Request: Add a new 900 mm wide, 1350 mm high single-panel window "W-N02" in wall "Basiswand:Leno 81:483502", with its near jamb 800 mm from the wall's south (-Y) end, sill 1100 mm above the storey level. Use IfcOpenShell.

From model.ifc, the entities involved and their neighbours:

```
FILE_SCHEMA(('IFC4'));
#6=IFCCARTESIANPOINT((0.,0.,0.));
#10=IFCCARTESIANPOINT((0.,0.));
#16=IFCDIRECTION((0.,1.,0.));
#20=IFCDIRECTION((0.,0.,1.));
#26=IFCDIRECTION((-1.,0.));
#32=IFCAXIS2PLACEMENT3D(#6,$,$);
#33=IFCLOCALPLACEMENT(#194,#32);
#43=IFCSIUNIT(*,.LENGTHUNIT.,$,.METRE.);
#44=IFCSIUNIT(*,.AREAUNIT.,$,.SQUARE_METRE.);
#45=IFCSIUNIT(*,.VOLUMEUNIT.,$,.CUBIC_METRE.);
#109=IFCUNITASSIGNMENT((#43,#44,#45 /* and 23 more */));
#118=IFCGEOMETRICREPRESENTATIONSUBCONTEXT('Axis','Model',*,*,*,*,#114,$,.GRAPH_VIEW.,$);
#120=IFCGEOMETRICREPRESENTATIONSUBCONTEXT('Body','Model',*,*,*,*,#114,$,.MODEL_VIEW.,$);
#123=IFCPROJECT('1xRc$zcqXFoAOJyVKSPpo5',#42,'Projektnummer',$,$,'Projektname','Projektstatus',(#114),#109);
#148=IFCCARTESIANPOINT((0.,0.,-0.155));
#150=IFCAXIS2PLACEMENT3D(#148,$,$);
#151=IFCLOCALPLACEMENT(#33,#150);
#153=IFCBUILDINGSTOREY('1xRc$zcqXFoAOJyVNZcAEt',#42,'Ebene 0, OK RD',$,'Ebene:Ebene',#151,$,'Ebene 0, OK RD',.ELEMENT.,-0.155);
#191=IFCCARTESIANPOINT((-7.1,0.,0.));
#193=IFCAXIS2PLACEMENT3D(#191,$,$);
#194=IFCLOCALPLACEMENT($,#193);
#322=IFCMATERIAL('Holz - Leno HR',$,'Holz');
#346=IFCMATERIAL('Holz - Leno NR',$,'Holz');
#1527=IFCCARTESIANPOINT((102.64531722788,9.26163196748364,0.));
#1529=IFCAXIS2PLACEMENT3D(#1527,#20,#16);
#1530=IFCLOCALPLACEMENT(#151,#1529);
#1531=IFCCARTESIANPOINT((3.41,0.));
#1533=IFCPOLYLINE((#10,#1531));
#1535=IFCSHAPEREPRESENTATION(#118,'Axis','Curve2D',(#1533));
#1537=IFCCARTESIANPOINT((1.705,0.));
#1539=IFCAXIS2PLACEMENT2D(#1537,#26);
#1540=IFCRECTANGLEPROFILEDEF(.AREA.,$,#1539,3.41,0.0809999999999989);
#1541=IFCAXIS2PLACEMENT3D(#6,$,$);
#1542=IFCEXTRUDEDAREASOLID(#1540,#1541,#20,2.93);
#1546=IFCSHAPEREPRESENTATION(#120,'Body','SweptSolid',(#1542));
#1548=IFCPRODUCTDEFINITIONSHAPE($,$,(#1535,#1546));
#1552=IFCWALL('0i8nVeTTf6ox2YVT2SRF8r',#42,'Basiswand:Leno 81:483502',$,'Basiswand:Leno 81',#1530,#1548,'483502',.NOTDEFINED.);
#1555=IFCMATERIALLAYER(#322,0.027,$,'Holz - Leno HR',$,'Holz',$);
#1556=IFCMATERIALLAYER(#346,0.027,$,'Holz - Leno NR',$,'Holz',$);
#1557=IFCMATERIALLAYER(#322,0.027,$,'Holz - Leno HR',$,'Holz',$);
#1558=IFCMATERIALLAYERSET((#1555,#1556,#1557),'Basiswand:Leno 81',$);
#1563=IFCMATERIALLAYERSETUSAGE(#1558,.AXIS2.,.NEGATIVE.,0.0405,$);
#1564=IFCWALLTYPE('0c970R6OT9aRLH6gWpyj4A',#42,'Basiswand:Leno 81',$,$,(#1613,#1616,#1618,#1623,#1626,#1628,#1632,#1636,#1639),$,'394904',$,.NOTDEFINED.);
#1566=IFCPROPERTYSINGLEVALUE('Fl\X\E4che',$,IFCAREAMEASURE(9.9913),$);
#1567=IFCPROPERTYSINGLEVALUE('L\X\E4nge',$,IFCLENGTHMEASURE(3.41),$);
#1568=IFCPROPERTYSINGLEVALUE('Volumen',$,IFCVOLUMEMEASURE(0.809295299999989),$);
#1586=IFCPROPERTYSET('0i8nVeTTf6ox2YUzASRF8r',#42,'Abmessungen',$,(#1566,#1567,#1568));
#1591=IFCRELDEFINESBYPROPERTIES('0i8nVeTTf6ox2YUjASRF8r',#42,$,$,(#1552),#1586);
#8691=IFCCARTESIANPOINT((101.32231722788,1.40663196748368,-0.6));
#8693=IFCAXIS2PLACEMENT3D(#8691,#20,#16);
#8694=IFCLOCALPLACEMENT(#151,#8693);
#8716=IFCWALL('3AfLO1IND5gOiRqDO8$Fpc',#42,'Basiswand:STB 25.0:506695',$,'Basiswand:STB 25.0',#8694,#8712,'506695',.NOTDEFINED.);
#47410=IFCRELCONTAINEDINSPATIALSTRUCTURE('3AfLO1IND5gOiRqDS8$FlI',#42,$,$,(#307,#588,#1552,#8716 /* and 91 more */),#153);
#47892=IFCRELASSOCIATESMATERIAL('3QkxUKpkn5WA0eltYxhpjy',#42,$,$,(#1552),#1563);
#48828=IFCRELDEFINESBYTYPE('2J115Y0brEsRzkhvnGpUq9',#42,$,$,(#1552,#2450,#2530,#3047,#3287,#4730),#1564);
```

```python
import numpy as np
import ifcopenshell
import ifcopenshell.api.feature
import ifcopenshell.api.geometry
import ifcopenshell.api.pset
import ifcopenshell.api.root
import ifcopenshell.api.spatial
import ifcopenshell.geom
import ifcopenshell.util.element
import ifcopenshell.util.placement
import ifcopenshell.util.representation
import ifcopenshell.util.shape
import ifcopenshell.util.unit

model = ifcopenshell.open("model.ifc")
unit_scale = ifcopenshell.util.unit.calculate_unit_scale(model)
area_scale = ifcopenshell.util.unit.calculate_unit_scale(model, "AREAUNIT")
volume_scale = ifcopenshell.util.unit.calculate_unit_scale(model, "VOLUMEUNIT")
settings = ifcopenshell.geom.settings()


def volume(element):
    """Net volume in cubic metres, openings subtracted."""
    shape = ifcopenshell.geom.create_shape(settings, element)
    return ifcopenshell.util.shape.get_volume(shape.geometry)


wall = model.by_id(1552)
storey = ifcopenshell.util.element.get_container(wall, ifc_class="IfcBuildingStorey")
context = ifcopenshell.util.representation.get_context(model, "Model", "Body", "MODEL_VIEW")
before = volume(wall)

width, height, from_end, sill = 0.9, 1.35, 0.8, 1.1  # metres

# The wall runs along its own X axis, and the end named is its -X end.
wall_shape = ifcopenshell.geom.create_shape(settings, wall)
x, y, z = ifcopenshell.util.shape.get_vertices(wall_shape.geometry).T
start = x.min() + from_end
face, thickness = float(y.min()), float(y.max() - y.min())
wall_matrix = ifcopenshell.util.placement.get_local_placement(wall.ObjectPlacement)
level = ifcopenshell.util.placement.get_local_placement(storey.ObjectPlacement)[2, 3]


def in_wall(x, y):
    """Placement at x, y metres in the wall's axes, at sill height."""
    matrix = wall_matrix.copy()
    matrix[:, 3] = wall_matrix @ np.array([x / unit_scale, y / unit_scale, 0.0, 1.0])
    matrix[2, 3] = level + sill / unit_scale
    return matrix


# Opening: a box that overshoots both wall faces by 50 mm.
opening = ifcopenshell.api.root.create_entity(model, ifc_class="IfcOpeningElement", predefined_type="OPENING")
box = ifcopenshell.api.geometry.add_wall_representation(
    model, context=context, length=width, height=height, thickness=thickness + 0.1
)
ifcopenshell.api.geometry.assign_representation(model, product=opening, representation=box)
ifcopenshell.api.geometry.edit_object_placement(model, product=opening, matrix=in_wall(start, face - 0.05), is_si=False)
ifcopenshell.api.feature.add_feature(model, feature=opening, element=wall)

window = ifcopenshell.api.root.create_entity(model, ifc_class="IfcWindow", name="W-N02", predefined_type="WINDOW")
window.OverallWidth, window.OverallHeight = width / unit_scale, height / unit_scale
window.PartitioningType = "SINGLE_PANEL"
body = ifcopenshell.api.geometry.add_window_representation(
    model,
    context=context,
    overall_width=window.OverallWidth,
    overall_height=window.OverallHeight,
    partition_type="SINGLE_PANEL",
)
ifcopenshell.api.geometry.assign_representation(model, product=window, representation=body)
ifcopenshell.api.spatial.assign_container(model, products=[window], relating_structure=storey)
ifcopenshell.api.feature.add_filling(model, opening=opening, element=window)

# Centre the window in the wall's thickness.
ifcopenshell.api.geometry.edit_object_placement(model, product=window, matrix=in_wall(start, face), is_si=False)
window_shape = ifcopenshell.geom.create_shape(settings, window)
depth = ifcopenshell.util.shape.get_vertices(window_shape.geometry)[:, 1]
offset = face + thickness / 2 - (depth.min() + depth.max()) / 2
ifcopenshell.api.geometry.edit_object_placement(model, product=window, matrix=in_wall(start, offset), is_si=False)

after = volume(wall)

# Update the wall's stored quantities.
pset = model.by_id(ifcopenshell.util.element.get_pset(wall, "Abmessungen", should_inherit=False)["id"])
ifcopenshell.api.pset.edit_pset(model, pset=pset, properties={
    "Fläche": model.create_entity("IfcAreaMeasure", after / thickness / area_scale),
    "Volumen": model.create_entity("IfcVolumeMeasure", after / volume_scale),
})

print(f"wall volume {before:.3f} -> {after:.3f} m3")

model.write("model_updated.ifc")
```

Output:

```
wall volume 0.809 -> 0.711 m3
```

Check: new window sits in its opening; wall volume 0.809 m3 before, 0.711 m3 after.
